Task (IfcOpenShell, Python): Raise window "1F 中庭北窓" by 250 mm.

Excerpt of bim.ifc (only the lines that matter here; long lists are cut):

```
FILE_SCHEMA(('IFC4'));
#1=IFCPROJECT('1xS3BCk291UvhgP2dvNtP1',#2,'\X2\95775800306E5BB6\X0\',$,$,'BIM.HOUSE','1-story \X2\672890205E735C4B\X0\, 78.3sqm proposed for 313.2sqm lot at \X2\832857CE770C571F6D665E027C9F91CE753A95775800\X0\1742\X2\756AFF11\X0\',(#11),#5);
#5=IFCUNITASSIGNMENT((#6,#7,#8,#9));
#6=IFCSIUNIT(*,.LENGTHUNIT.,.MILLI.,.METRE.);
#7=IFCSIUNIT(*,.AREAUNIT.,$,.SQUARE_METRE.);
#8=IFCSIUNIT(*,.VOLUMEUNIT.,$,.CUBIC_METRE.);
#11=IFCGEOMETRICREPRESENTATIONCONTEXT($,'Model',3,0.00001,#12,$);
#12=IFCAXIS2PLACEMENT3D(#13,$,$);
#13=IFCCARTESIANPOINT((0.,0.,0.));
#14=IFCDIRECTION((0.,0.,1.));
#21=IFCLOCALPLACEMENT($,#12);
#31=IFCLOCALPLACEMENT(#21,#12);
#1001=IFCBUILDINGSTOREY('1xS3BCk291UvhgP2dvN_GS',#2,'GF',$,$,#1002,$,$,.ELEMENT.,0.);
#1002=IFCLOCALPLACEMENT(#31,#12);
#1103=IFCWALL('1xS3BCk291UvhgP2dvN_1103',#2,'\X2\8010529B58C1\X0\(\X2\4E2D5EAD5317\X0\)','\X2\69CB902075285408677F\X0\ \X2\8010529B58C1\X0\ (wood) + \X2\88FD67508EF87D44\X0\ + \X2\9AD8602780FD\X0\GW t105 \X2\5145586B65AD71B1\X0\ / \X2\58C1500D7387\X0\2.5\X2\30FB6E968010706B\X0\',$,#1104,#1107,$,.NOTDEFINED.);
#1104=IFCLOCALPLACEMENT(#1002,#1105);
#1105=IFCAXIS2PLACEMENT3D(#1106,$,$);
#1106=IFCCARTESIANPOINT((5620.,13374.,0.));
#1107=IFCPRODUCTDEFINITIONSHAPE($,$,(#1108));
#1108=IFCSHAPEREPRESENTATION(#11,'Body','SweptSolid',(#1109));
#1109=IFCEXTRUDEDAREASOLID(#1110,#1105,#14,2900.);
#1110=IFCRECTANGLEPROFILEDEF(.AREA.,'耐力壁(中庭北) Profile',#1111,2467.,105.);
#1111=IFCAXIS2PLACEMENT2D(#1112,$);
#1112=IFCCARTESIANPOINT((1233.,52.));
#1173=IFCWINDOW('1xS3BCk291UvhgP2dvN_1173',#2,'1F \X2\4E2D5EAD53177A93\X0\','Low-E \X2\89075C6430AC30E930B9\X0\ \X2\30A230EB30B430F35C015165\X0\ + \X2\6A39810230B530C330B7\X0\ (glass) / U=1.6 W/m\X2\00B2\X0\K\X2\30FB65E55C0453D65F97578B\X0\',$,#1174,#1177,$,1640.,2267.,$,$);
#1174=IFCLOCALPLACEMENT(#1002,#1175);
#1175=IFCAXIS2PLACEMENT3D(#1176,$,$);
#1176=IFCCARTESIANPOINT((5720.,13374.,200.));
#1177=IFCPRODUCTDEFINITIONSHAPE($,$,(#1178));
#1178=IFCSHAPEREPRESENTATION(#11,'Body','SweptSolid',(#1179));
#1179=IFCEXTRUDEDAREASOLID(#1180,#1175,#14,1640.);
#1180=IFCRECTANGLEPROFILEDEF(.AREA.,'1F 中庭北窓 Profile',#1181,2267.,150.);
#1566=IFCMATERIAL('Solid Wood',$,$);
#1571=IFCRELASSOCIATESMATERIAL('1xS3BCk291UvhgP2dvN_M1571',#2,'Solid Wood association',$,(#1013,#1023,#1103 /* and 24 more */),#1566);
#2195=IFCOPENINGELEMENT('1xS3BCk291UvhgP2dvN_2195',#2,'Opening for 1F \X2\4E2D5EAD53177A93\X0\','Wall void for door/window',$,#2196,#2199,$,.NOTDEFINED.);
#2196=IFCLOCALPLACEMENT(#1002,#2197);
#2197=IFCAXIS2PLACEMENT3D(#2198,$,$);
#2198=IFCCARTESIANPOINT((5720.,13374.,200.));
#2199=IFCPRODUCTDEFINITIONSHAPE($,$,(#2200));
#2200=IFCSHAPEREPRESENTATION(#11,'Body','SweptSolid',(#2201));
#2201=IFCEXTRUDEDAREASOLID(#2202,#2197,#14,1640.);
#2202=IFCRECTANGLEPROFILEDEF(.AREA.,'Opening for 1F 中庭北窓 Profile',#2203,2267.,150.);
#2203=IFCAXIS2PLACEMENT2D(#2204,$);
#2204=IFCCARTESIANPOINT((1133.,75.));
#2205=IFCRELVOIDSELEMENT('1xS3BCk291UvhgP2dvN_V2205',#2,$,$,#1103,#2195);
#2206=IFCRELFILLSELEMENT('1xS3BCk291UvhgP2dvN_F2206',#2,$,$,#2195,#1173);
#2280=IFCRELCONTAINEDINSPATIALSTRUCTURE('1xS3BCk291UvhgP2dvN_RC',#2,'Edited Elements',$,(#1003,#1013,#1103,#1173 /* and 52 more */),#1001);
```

```python
import numpy as np
import ifcopenshell
import ifcopenshell.api.geometry
import ifcopenshell.util.placement
import ifcopenshell.util.unit

model = ifcopenshell.open("bim.ifc")
unit_scale = ifcopenshell.util.unit.calculate_unit_scale(model)

window = model.by_guid("1xS3BCk291UvhgP2dvN_1173")
opening = window.FillsVoids[0].RelatingOpeningElement
dz = 0.25 / unit_scale

shift = np.array([0.0, 0.0, dz])
# The window is not placed relative to its opening, so move both.
for product in (opening, window):
    matrix = ifcopenshell.util.placement.get_local_placement(product.ObjectPlacement)
    matrix[:3, 3] += shift
    ifcopenshell.api.geometry.edit_object_placement(model, product=product, matrix=matrix, is_si=False)

print(f"moved by {dz * unit_scale:+.3f} m")

model.write("bim_rev.ifc")
```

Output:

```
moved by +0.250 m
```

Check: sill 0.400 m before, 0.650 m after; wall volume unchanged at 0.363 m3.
